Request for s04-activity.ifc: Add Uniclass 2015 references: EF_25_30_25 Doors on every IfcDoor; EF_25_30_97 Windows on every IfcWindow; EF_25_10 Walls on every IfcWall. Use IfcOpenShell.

First a look at what the model holds.

```python
import ifcopenshell

model = ifcopenshell.open("s04-activity.ifc")
print(model.schema)
print("classifications:", [c.Name for c in model.by_type("IfcClassification")])
for ifc_class in ("IfcDoor", "IfcRoof", "IfcStair", "IfcWall", "IfcWindow"):
    print(ifc_class, len(model.by_type(ifc_class)))
```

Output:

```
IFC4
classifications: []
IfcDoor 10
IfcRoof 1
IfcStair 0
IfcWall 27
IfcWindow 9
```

```python
import ifcopenshell
import ifcopenshell.api.classification

model = ifcopenshell.open("s04-activity.ifc")

system = ifcopenshell.api.classification.add_classification(model, classification="Uniclass 2015")

codes = {
    "IfcDoor": ("EF_25_30_25", "Doors"),
    "IfcWindow": ("EF_25_30_97", "Windows"),
    "IfcWall": ("EF_25_10", "Walls"),
}
for ifc_class, (code, name) in codes.items():
    products = model.by_type(ifc_class)
    ifcopenshell.api.classification.add_reference(
        model, products=products, classification=system, identification=code, name=name
    )
    print(code, len(products))

model.write("s04-activity_edited.ifc")
```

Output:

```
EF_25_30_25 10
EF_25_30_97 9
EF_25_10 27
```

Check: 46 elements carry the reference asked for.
